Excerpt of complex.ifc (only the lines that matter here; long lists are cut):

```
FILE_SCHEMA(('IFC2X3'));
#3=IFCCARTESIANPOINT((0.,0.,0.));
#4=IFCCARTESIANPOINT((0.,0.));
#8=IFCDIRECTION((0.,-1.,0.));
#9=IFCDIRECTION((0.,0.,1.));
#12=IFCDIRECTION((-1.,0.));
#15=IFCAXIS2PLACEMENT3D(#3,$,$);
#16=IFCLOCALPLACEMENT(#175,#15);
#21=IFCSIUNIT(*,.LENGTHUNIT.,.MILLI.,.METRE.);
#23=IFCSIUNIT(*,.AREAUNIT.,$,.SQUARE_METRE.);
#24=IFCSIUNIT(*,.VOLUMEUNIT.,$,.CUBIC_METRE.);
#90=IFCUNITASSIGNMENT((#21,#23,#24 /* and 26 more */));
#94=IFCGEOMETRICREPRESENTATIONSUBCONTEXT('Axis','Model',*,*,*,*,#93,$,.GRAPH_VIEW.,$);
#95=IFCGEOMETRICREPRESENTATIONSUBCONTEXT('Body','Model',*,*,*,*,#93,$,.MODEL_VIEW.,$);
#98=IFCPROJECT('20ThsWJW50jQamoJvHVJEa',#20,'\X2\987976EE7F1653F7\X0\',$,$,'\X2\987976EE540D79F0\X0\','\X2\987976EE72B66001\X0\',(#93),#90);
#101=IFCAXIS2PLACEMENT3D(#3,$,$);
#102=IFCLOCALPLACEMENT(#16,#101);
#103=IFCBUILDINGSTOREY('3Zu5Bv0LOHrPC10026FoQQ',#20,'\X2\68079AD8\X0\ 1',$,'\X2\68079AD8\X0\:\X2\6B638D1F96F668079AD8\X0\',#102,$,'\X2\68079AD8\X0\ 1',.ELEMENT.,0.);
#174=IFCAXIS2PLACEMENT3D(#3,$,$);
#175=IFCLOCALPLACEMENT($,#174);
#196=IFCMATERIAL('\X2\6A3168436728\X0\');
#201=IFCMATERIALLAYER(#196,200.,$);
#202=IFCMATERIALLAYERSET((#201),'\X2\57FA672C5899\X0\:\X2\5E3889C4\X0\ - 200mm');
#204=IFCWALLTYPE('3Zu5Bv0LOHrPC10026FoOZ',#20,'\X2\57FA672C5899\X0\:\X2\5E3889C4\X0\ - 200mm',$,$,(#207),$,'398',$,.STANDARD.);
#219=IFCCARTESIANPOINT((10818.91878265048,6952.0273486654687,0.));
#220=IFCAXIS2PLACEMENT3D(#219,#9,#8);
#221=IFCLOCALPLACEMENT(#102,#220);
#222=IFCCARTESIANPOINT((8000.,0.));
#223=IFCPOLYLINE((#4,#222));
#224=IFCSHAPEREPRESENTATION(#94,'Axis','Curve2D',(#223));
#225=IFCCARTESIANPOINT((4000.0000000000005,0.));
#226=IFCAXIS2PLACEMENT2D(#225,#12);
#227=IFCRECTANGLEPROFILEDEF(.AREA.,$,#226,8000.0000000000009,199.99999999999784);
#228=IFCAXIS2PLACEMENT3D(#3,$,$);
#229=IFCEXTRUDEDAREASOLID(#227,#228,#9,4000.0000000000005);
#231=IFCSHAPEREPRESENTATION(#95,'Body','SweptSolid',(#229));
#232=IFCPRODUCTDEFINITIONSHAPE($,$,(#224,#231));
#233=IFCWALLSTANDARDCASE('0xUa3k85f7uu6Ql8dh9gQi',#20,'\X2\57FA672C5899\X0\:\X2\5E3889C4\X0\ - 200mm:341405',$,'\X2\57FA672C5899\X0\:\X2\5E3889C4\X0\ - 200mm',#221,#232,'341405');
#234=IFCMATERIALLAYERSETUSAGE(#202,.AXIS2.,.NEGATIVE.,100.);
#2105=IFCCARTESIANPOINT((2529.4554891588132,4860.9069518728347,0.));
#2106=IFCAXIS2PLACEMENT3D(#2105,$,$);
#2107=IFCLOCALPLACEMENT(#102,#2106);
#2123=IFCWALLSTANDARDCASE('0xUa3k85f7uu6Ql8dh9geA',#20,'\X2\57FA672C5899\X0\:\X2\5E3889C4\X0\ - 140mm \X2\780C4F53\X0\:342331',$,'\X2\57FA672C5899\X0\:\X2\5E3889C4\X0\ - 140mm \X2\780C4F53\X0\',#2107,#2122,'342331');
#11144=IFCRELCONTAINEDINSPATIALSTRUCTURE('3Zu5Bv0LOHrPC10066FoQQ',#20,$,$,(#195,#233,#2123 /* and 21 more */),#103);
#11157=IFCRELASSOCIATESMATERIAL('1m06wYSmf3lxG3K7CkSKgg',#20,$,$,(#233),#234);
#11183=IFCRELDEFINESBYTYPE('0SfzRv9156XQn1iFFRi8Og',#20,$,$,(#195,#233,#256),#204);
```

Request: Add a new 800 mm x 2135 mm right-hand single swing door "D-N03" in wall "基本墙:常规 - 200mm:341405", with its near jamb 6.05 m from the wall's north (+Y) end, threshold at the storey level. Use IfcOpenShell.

```python
import numpy as np
import ifcopenshell
import ifcopenshell.api.feature
import ifcopenshell.api.geometry
import ifcopenshell.api.root
import ifcopenshell.api.spatial
import ifcopenshell.api.type
import ifcopenshell.geom
import ifcopenshell.util.element
import ifcopenshell.util.placement
import ifcopenshell.util.representation
import ifcopenshell.util.shape
import ifcopenshell.util.unit

model = ifcopenshell.open("complex.ifc")
unit_scale = ifcopenshell.util.unit.calculate_unit_scale(model)
settings = ifcopenshell.geom.settings()


def volume(element):
    """Net volume in cubic metres, openings subtracted."""
    shape = ifcopenshell.geom.create_shape(settings, element)
    return ifcopenshell.util.shape.get_volume(shape.geometry)


wall = model.by_guid("0xUa3k85f7uu6Ql8dh9gQi")
storey = ifcopenshell.util.element.get_container(wall, ifc_class="IfcBuildingStorey")
context = ifcopenshell.util.representation.get_context(model, "Model", "Body", "MODEL_VIEW")
before = volume(wall)

width, height, from_end, sill = 0.8, 2.135, 6.05, 0.0  # metres

# The wall runs along its own X axis, and the end named is its -X end.
wall_shape = ifcopenshell.geom.create_shape(settings, wall)
x, y, z = ifcopenshell.util.shape.get_vertices(wall_shape.geometry).T
start = x.min() + from_end
face, thickness = float(y.min()), float(y.max() - y.min())
wall_matrix = ifcopenshell.util.placement.get_local_placement(wall.ObjectPlacement)
level = ifcopenshell.util.placement.get_local_placement(storey.ObjectPlacement)[2, 3]


def in_wall(x, y):
    """Placement at x, y metres in the wall's axes, at sill height."""
    matrix = wall_matrix.copy()
    matrix[:, 3] = wall_matrix @ np.array([x / unit_scale, y / unit_scale, 0.0, 1.0])
    matrix[2, 3] = level + sill / unit_scale
    return matrix


# Opening: a box that overshoots both wall faces by 50 mm.
opening = ifcopenshell.api.root.create_entity(model, ifc_class="IfcOpeningElement")
box = ifcopenshell.api.geometry.add_wall_representation(
    model, context=context, length=width, height=height, thickness=thickness + 0.1
)
ifcopenshell.api.geometry.assign_representation(model, product=opening, representation=box)
ifcopenshell.api.geometry.edit_object_placement(model, product=opening, matrix=in_wall(start, face - 0.05), is_si=False)
ifcopenshell.api.feature.add_feature(model, feature=opening, element=wall)

door = ifcopenshell.api.root.create_entity(model, ifc_class="IfcDoor", name="D-N03")
door.OverallWidth, door.OverallHeight = width / unit_scale, height / unit_scale
body = ifcopenshell.api.geometry.add_door_representation(
    model,
    context=context,
    overall_width=door.OverallWidth,
    overall_height=door.OverallHeight,
    operation_type="SINGLE_SWING_RIGHT",
    lining_properties={"LiningDepth": thickness / unit_scale, "ThresholdDepth": thickness / unit_scale},
)
ifcopenshell.api.geometry.assign_representation(model, product=door, representation=body)
ifcopenshell.api.spatial.assign_container(model, products=[door], relating_structure=storey)
fills = ifcopenshell.api.feature.add_filling(model, opening=opening, element=door)
fills.OwnerHistory = door.OwnerHistory  # required in IFC2X3

# IFC2X3 keeps the operation on the door style.
style = ifcopenshell.api.root.create_entity(model, ifc_class="IfcDoorStyle", name="D-N03")
style.OperationType, style.ConstructionType = "SINGLE_SWING_RIGHT", "NOTDEFINED"
style.ParameterTakesPrecedence = style.Sizeable = False
ifcopenshell.api.type.assign_type(model, related_objects=[door], relating_type=style)

# The lining spans the wall, so the door starts at the wall face.
ifcopenshell.api.geometry.edit_object_placement(model, product=door, matrix=in_wall(start, face), is_si=False)

after = volume(wall)

print(f"wall volume {before:.3f} -> {after:.3f} m3")

model.write("complex_v2.ifc")
```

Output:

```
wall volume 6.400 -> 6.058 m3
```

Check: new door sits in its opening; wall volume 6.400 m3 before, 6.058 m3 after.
